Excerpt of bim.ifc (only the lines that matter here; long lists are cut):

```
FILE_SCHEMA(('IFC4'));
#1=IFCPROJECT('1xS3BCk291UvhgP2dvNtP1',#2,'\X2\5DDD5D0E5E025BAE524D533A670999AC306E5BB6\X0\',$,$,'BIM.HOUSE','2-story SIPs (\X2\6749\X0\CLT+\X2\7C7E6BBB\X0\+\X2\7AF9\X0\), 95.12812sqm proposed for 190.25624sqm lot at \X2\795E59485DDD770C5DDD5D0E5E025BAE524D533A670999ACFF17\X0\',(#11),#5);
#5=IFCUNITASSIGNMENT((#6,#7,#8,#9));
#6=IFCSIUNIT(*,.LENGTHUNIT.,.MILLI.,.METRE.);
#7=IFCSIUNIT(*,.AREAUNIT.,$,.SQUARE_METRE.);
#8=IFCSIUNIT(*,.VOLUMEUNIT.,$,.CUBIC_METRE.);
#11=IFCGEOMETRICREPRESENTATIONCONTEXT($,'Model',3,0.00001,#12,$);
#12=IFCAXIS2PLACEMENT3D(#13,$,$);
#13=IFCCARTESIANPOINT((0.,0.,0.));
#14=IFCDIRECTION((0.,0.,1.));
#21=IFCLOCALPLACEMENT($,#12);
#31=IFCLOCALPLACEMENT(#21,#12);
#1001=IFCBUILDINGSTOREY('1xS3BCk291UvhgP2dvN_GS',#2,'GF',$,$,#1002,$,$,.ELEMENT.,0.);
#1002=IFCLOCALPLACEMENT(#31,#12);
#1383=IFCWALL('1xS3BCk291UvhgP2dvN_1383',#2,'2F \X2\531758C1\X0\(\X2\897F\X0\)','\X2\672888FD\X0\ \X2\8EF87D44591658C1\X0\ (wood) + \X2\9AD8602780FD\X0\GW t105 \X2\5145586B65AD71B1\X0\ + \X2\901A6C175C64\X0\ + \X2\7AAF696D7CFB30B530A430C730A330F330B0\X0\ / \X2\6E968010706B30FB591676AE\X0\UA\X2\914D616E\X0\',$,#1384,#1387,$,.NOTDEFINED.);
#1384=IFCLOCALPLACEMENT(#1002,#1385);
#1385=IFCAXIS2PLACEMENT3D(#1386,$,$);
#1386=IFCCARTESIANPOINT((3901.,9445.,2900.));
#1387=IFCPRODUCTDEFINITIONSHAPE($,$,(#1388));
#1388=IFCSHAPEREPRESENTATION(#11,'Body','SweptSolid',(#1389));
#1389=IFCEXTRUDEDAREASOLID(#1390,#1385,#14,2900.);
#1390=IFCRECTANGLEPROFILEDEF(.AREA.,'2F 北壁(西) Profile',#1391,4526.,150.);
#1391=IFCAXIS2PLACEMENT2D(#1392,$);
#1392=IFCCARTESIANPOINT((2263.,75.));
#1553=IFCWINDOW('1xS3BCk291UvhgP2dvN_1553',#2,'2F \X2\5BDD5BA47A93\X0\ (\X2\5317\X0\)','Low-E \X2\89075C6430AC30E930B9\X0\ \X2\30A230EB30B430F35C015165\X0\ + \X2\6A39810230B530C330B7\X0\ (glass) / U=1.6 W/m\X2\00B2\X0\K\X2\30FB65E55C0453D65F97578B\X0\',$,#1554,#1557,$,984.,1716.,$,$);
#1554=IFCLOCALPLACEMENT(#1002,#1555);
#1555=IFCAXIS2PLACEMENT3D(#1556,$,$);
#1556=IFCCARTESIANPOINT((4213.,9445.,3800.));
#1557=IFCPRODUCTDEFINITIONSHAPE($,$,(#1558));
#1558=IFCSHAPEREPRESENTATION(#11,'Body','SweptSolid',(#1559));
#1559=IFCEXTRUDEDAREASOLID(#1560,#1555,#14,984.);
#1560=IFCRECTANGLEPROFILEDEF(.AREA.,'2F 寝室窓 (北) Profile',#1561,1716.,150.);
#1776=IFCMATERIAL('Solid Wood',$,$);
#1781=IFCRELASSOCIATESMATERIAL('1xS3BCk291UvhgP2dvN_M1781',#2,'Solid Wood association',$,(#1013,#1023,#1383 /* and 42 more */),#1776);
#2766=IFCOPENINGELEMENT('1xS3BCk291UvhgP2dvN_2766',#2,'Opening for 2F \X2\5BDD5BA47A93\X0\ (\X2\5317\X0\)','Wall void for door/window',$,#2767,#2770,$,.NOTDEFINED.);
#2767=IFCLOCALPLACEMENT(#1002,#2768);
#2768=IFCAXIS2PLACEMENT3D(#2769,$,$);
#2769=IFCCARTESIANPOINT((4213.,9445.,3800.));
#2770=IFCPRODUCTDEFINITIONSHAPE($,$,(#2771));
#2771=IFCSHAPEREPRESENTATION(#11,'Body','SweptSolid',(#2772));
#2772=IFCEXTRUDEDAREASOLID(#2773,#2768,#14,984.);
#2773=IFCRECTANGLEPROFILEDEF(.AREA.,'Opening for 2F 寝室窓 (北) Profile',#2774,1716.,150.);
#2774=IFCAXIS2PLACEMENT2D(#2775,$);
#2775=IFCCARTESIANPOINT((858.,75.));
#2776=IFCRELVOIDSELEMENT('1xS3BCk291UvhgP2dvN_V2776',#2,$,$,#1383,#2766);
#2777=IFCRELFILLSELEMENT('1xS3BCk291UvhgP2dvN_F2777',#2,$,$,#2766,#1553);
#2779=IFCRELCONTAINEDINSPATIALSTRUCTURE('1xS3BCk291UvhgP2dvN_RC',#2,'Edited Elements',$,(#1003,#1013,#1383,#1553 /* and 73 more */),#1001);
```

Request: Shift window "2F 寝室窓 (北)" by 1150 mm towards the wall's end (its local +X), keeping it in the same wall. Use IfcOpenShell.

```python
import ifcopenshell
import ifcopenshell.api.geometry
import ifcopenshell.util.placement
import ifcopenshell.util.unit

model = ifcopenshell.open("bim.ifc")
unit_scale = ifcopenshell.util.unit.calculate_unit_scale(model)

window = model.by_id(1553)
opening = window.FillsVoids[0].RelatingOpeningElement
wall = opening.VoidsElements[0].RelatingBuildingElement

wall_matrix = ifcopenshell.util.placement.get_local_placement(wall.ObjectPlacement)
shift = wall_matrix[:3, 0] * 1.15 / unit_scale
before = ifcopenshell.util.placement.get_local_placement(window.ObjectPlacement)[:3, 3].copy()

# The window is not placed relative to its opening, so move both.
for product in (opening, window):
    matrix = ifcopenshell.util.placement.get_local_placement(product.ObjectPlacement)
    matrix[:3, 3] += shift
    ifcopenshell.api.geometry.edit_object_placement(model, product=product, matrix=matrix, is_si=False)

after = ifcopenshell.util.placement.get_local_placement(window.ObjectPlacement)[:3, 3]
print("window moved by", (after - before).round(3) + 0.0)

model.write("bim_v2.ifc")
```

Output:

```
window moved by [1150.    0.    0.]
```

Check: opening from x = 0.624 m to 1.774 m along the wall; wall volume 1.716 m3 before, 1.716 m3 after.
